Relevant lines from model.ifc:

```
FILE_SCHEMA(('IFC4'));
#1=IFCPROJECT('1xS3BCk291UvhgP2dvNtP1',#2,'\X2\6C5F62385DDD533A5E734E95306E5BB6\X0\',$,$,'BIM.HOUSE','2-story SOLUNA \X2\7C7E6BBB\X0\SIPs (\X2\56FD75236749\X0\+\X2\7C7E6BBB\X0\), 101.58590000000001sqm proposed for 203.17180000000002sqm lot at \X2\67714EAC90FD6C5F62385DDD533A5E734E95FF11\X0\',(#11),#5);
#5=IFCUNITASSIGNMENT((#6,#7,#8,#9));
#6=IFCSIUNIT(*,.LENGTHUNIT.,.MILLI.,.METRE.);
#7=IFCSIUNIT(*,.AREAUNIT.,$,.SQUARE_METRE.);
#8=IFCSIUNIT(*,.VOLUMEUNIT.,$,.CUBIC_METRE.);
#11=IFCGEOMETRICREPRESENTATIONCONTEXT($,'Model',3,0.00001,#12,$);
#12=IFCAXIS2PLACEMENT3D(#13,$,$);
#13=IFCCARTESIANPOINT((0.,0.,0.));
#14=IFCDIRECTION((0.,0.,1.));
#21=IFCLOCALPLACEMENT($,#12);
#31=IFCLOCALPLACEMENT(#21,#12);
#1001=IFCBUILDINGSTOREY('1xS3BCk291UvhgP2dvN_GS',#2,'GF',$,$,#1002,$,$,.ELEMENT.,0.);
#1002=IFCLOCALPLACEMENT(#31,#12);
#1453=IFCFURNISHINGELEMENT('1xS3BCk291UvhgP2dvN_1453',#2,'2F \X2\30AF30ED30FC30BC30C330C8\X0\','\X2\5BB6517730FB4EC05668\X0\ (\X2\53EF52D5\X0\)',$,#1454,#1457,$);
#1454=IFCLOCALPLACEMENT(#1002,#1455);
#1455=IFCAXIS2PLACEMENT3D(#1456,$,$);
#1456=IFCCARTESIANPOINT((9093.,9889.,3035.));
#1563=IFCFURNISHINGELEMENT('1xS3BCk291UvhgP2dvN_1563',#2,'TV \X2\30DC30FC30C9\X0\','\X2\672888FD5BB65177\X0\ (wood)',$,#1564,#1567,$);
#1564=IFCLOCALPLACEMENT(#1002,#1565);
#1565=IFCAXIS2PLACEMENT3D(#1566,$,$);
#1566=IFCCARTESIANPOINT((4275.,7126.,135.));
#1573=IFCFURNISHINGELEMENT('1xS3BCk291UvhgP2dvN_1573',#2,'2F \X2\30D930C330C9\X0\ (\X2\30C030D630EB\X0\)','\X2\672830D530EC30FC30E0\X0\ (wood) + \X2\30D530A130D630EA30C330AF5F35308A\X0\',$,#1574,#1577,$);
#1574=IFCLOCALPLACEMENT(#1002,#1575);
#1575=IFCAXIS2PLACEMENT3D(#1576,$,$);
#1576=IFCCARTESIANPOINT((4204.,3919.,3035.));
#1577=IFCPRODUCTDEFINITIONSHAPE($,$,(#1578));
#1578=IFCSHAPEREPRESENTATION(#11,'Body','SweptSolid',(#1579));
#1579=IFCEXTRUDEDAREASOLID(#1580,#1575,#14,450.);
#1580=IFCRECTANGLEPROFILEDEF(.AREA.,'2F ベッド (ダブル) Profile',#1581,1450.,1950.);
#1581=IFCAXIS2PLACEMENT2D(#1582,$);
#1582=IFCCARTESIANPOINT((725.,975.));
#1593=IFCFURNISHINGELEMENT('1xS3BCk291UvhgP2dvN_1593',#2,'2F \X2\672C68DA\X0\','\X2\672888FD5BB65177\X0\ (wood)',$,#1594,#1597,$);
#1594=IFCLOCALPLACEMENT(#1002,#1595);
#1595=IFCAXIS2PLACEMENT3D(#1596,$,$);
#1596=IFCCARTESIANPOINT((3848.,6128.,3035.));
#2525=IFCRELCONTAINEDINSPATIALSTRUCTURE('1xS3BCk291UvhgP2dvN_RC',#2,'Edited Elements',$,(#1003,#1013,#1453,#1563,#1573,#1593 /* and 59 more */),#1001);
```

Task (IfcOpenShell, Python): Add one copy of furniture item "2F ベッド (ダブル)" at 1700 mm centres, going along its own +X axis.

```python
import ifcopenshell
import ifcopenshell.api.geometry
import ifcopenshell.api.root
import ifcopenshell.util.element
import ifcopenshell.util.placement

model = ifcopenshell.open("model.ifc")


def reuse_history(source, copy):
    """copy_class also copies each property set's owner history, people and application; keep the originals."""
    for rel in copy.IsDefinedBy:
        if rel.is_a("IfcRelDefinesByProperties") and (history := rel.RelatingPropertyDefinition.OwnerHistory):
            rel.RelatingPropertyDefinition.OwnerHistory = source.OwnerHistory
            ifcopenshell.util.element.remove_deep2(model, history)


source = model.by_guid("1xS3BCk291UvhgP2dvN_1573")
base = ifcopenshell.util.placement.get_local_placement(source.ObjectPlacement)
step = base[:3, 0] * 1700.0

for i in range(1, 2):
    copy = ifcopenshell.api.root.copy_class(model, product=source)
    copy.Representation = ifcopenshell.util.element.copy_deep(
        model, source.Representation, exclude=["IfcGeometricRepresentationContext", "IfcRepresentationMap"]
    )
    reuse_history(source, copy)
    matrix = base.copy()
    matrix[:3, 3] += i * step
    print("added at", matrix[:3, 3].round(3) + 0.0)
    ifcopenshell.api.geometry.edit_object_placement(model, product=copy, matrix=matrix, is_si=False)

model.write("model_edited.ifc")
```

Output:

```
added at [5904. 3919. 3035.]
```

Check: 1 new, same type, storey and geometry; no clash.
